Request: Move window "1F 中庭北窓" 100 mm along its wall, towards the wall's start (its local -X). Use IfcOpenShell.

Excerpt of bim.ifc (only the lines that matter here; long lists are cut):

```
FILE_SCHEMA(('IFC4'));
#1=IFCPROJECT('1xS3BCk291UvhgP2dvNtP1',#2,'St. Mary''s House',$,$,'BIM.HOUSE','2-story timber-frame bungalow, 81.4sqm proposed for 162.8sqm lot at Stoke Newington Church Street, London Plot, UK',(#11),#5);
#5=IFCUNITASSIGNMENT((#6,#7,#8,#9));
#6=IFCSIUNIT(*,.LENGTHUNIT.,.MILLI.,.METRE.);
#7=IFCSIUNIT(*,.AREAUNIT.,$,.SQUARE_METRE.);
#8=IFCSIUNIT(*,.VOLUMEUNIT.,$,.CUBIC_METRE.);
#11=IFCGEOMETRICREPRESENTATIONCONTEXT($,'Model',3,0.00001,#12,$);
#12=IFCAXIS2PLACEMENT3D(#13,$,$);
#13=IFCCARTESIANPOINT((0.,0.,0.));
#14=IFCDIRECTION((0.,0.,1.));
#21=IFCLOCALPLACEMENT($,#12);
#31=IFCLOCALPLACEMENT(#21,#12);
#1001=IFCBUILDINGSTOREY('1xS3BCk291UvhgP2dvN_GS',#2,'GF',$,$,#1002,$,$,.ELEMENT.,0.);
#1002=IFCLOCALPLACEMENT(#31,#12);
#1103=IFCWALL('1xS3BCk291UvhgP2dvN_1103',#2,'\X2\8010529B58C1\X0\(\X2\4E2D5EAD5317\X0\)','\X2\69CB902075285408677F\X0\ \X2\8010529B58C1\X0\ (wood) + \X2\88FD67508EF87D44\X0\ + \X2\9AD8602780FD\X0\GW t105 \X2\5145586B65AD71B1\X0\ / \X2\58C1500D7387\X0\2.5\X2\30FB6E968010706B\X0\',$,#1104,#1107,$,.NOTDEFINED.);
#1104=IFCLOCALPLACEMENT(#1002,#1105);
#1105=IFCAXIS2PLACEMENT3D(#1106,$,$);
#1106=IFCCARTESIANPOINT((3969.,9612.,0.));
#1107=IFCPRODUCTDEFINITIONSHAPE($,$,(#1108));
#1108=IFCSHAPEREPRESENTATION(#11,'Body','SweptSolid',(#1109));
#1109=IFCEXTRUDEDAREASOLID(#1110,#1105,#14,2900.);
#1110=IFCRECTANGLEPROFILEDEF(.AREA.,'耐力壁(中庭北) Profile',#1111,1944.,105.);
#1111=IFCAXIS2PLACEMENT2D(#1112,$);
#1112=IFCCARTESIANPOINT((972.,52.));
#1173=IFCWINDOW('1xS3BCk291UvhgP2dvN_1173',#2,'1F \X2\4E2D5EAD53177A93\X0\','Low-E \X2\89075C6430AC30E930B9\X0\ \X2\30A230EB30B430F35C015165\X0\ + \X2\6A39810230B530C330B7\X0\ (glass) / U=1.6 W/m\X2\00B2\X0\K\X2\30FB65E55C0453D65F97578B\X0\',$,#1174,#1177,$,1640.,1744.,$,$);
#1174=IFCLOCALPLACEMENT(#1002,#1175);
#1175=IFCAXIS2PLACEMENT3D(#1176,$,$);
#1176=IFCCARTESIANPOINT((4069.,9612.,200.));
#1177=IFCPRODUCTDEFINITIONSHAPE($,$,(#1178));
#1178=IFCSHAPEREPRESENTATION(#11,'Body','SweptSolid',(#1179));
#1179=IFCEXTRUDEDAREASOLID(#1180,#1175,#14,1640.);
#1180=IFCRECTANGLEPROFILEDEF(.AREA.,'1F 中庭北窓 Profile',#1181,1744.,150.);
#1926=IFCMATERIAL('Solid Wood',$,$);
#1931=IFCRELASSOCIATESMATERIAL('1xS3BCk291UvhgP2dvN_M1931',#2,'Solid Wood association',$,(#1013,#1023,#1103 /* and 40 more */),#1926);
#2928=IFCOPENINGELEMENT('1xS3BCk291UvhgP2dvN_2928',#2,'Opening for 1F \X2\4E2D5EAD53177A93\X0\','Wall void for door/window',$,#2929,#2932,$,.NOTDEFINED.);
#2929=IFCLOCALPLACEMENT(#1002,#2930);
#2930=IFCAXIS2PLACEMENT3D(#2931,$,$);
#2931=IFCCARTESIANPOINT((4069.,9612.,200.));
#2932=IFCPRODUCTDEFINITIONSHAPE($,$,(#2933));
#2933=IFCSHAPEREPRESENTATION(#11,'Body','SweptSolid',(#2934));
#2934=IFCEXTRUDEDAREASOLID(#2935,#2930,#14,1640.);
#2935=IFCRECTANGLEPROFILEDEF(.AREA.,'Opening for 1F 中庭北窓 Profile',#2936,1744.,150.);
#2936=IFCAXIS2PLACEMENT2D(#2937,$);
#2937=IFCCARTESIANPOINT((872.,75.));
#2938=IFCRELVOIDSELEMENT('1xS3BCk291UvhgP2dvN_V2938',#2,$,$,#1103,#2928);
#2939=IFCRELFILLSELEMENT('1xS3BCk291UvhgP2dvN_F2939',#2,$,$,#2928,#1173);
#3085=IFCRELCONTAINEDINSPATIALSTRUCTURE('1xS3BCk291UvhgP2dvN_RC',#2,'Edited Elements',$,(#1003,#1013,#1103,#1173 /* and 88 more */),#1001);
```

```python
import ifcopenshell
import ifcopenshell.api.geometry
import ifcopenshell.util.placement
import ifcopenshell.util.unit

model = ifcopenshell.open("bim.ifc")
unit_scale = ifcopenshell.util.unit.calculate_unit_scale(model)

window = model.by_guid("1xS3BCk291UvhgP2dvN_1173")
opening = window.FillsVoids[0].RelatingOpeningElement
wall = opening.VoidsElements[0].RelatingBuildingElement

wall_matrix = ifcopenshell.util.placement.get_local_placement(wall.ObjectPlacement)
shift = wall_matrix[:3, 0] * -0.1 / unit_scale
before = ifcopenshell.util.placement.get_local_placement(window.ObjectPlacement)[:3, 3].copy()

# The window is not placed relative to its opening, so move both.
for product in (opening, window):
    matrix = ifcopenshell.util.placement.get_local_placement(product.ObjectPlacement)
    matrix[:3, 3] += shift
    ifcopenshell.api.geometry.edit_object_placement(model, product=product, matrix=matrix, is_si=False)

after = ifcopenshell.util.placement.get_local_placement(window.ObjectPlacement)[:3, 3]
print("window moved by", (after - before).round(3) + 0.0)

model.write("bim_updated.ifc")
```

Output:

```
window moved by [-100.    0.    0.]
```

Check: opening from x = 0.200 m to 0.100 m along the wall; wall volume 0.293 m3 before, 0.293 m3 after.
